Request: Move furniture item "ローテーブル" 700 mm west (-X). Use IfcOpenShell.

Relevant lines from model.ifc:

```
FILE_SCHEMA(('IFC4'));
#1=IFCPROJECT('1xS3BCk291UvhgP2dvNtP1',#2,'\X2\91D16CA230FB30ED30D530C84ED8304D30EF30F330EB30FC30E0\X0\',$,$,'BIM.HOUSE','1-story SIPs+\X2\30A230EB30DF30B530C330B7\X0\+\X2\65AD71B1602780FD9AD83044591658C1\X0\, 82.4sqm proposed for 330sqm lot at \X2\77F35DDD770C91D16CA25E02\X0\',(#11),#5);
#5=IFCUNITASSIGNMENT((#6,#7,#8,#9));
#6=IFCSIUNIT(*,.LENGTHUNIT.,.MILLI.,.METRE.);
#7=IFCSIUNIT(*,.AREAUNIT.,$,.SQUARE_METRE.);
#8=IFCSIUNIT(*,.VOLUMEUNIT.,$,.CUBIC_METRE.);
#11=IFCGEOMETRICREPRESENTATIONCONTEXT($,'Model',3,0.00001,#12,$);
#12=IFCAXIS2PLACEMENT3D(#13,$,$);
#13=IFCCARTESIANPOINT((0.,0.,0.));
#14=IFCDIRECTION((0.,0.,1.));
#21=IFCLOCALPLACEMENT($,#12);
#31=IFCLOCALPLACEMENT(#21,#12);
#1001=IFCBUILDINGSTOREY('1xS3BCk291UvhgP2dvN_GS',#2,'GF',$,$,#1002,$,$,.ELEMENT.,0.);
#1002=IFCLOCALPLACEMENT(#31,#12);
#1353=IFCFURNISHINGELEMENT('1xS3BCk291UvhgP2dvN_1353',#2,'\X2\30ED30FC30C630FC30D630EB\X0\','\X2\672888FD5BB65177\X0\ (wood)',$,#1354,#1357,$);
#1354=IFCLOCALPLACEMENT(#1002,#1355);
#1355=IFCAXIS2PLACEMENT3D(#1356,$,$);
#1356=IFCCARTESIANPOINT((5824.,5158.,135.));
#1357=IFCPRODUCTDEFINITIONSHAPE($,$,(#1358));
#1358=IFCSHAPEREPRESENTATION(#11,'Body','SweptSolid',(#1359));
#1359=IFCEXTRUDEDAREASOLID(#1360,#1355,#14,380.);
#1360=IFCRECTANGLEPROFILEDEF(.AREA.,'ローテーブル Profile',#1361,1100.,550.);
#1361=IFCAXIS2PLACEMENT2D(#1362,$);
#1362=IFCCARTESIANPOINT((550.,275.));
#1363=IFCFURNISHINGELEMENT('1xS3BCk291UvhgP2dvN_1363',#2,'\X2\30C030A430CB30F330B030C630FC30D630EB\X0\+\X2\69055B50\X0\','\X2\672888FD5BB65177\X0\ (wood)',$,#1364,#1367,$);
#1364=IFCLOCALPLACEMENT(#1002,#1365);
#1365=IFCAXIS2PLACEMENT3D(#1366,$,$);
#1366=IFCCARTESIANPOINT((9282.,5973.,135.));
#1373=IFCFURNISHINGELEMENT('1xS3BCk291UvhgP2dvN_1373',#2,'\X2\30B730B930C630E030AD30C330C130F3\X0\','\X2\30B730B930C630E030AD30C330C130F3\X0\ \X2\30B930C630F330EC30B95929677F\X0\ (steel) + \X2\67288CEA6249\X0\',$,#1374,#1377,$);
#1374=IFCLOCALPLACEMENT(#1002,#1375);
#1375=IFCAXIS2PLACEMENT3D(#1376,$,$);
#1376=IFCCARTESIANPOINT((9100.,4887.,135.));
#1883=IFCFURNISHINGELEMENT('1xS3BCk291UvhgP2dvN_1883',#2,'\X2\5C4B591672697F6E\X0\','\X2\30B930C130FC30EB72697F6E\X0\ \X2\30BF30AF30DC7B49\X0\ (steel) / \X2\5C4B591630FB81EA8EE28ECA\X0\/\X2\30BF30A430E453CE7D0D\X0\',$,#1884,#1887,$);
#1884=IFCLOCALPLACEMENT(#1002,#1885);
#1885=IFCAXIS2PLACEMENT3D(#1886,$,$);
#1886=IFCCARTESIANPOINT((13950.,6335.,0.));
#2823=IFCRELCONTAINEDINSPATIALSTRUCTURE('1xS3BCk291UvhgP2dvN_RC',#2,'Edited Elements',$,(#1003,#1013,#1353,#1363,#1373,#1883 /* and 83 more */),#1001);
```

```python
import ifcopenshell
import ifcopenshell.api.geometry
import ifcopenshell.util.placement

model = ifcopenshell.open("model.ifc")

item = model.by_id(1353)
matrix = ifcopenshell.util.placement.get_local_placement(item.ObjectPlacement)
matrix[0, 3] -= 700.0
ifcopenshell.api.geometry.edit_object_placement(model, product=item, matrix=matrix, is_si=False)

print(ifcopenshell.util.placement.get_local_placement(item.ObjectPlacement).round(3) + 0.0)

model.write("model_edited.ifc")
```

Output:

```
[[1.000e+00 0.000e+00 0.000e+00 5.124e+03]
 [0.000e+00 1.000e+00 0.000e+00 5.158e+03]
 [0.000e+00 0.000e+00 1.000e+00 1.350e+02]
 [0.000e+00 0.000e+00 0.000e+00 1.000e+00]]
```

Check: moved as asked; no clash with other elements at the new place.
